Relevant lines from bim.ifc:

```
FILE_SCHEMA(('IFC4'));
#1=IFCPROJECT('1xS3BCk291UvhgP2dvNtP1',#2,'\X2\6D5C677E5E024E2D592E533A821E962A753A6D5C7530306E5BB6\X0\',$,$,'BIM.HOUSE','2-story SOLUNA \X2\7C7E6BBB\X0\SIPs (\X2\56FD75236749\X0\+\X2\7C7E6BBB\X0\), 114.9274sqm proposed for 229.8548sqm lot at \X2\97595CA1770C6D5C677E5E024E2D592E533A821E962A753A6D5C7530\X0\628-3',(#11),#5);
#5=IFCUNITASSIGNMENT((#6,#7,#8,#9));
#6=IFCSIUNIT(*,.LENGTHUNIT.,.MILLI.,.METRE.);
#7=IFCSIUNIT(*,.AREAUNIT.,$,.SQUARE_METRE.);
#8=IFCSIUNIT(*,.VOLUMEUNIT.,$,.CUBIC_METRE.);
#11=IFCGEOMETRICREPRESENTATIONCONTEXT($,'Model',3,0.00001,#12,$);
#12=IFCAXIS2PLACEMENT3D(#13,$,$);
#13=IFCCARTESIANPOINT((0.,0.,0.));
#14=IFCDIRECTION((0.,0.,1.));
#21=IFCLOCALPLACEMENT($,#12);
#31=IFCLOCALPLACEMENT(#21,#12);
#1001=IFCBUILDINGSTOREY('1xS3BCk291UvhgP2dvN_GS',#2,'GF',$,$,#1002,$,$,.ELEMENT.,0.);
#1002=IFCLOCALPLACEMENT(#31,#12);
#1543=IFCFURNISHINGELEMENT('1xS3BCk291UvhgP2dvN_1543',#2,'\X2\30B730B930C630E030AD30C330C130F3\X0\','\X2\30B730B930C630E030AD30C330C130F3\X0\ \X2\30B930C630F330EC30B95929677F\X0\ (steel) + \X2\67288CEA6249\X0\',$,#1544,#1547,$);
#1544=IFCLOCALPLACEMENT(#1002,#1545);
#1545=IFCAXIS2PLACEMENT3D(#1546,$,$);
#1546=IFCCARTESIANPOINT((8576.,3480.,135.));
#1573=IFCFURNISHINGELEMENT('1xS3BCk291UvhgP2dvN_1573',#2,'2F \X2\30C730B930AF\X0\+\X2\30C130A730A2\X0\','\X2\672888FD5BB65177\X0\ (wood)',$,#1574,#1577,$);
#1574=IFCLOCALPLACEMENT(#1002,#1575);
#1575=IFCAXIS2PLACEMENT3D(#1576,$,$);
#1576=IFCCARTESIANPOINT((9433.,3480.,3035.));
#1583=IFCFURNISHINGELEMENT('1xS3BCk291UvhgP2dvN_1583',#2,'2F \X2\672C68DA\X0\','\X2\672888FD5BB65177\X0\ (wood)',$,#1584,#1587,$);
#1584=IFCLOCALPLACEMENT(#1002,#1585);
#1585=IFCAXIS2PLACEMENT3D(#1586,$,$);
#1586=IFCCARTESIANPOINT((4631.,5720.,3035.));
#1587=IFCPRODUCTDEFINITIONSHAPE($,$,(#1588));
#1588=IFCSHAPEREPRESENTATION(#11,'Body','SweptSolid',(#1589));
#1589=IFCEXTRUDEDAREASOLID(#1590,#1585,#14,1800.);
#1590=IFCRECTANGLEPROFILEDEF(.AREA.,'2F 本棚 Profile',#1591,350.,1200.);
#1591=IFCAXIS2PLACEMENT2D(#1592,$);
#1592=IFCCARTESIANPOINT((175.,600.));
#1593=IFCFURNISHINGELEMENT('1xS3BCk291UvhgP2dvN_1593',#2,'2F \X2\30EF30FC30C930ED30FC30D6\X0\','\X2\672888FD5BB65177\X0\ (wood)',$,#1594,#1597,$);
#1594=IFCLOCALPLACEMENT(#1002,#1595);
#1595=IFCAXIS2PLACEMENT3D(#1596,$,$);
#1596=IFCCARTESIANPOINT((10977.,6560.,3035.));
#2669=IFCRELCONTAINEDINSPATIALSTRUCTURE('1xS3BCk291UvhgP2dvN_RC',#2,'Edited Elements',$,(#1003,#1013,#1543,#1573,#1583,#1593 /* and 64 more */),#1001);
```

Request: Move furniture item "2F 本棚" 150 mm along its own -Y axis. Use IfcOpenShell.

```python
import ifcopenshell
import ifcopenshell.api.geometry
import ifcopenshell.util.placement
import ifcopenshell.util.unit

model = ifcopenshell.open("bim.ifc")
unit_scale = ifcopenshell.util.unit.calculate_unit_scale(model)

item = model.by_id(1583)
matrix = ifcopenshell.util.placement.get_local_placement(item.ObjectPlacement)
matrix[:3, 3] -= matrix[:3, 1] * 0.15 / unit_scale
ifcopenshell.api.geometry.edit_object_placement(model, product=item, matrix=matrix, is_si=False)

print(ifcopenshell.util.placement.get_local_placement(item.ObjectPlacement).round(3) + 0.0)

model.write("bim_rev.ifc")
```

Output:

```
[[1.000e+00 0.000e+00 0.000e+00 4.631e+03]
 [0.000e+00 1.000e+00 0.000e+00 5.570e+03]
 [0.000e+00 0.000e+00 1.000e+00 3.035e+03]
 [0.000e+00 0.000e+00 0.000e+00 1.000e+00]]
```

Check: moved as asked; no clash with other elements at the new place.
